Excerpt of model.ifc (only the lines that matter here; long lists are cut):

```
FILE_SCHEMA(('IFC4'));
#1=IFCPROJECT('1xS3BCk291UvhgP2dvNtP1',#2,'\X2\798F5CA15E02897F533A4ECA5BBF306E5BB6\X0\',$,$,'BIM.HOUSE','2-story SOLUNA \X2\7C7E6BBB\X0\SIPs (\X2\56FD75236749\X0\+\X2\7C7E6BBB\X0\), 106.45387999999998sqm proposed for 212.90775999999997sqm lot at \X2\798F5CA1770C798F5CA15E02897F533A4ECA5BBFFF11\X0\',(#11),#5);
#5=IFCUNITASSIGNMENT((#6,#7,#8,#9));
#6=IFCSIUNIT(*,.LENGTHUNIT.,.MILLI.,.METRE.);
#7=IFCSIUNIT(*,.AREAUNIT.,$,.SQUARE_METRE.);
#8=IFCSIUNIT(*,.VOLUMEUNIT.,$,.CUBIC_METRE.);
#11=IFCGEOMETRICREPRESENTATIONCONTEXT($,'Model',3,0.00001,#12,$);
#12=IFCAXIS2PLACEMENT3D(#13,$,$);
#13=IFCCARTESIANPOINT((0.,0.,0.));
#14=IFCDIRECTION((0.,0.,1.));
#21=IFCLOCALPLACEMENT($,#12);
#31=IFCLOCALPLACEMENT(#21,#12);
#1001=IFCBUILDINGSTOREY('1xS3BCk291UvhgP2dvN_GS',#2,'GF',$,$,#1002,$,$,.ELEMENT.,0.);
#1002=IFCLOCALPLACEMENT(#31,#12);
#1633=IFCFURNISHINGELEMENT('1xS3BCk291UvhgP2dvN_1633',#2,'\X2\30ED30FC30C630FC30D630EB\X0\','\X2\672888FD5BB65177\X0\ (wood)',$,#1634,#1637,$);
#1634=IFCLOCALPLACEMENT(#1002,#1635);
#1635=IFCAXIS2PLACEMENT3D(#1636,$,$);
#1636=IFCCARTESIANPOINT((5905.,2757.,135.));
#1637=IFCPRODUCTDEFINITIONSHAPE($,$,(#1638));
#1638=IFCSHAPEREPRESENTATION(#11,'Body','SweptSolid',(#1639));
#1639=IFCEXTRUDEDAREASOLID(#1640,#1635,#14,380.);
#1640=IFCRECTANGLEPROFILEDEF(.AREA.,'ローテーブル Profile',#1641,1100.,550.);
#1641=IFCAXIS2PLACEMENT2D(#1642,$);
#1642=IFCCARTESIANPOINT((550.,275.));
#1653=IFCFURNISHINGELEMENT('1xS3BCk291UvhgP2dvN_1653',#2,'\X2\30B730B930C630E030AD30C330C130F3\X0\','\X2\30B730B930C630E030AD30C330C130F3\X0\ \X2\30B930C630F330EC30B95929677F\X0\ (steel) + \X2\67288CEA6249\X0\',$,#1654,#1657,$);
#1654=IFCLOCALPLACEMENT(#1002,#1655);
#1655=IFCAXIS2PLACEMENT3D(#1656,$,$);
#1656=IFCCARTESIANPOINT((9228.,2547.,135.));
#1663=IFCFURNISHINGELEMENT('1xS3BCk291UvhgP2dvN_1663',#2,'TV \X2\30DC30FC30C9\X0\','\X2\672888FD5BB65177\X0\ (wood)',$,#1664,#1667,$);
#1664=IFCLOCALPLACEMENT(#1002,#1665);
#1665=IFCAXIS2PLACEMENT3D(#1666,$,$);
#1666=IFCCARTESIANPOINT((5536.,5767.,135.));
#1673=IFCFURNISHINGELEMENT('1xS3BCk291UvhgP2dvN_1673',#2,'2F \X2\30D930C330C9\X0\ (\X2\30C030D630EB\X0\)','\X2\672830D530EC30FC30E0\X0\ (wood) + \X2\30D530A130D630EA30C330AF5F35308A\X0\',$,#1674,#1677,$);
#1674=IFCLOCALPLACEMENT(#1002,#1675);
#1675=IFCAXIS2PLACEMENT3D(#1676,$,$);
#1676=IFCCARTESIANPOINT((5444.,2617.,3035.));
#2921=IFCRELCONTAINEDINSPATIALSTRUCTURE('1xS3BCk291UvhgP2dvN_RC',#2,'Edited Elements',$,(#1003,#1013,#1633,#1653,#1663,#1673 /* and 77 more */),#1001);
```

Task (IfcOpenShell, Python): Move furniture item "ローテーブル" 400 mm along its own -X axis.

```python
import ifcopenshell
import ifcopenshell.api.geometry
import ifcopenshell.util.placement
import ifcopenshell.util.unit

model = ifcopenshell.open("model.ifc")
unit_scale = ifcopenshell.util.unit.calculate_unit_scale(model)

item = model.by_guid("1xS3BCk291UvhgP2dvN_1633")
matrix = ifcopenshell.util.placement.get_local_placement(item.ObjectPlacement)
matrix[:3, 3] -= matrix[:3, 0] * 0.4 / unit_scale
ifcopenshell.api.geometry.edit_object_placement(model, product=item, matrix=matrix, is_si=False)

print(ifcopenshell.util.placement.get_local_placement(item.ObjectPlacement).round(3) + 0.0)

model.write("model_rev.ifc")
```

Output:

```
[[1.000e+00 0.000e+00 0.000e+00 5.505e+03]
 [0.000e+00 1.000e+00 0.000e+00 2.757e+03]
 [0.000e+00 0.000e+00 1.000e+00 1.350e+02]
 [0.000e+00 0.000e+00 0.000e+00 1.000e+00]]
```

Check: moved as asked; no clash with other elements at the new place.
